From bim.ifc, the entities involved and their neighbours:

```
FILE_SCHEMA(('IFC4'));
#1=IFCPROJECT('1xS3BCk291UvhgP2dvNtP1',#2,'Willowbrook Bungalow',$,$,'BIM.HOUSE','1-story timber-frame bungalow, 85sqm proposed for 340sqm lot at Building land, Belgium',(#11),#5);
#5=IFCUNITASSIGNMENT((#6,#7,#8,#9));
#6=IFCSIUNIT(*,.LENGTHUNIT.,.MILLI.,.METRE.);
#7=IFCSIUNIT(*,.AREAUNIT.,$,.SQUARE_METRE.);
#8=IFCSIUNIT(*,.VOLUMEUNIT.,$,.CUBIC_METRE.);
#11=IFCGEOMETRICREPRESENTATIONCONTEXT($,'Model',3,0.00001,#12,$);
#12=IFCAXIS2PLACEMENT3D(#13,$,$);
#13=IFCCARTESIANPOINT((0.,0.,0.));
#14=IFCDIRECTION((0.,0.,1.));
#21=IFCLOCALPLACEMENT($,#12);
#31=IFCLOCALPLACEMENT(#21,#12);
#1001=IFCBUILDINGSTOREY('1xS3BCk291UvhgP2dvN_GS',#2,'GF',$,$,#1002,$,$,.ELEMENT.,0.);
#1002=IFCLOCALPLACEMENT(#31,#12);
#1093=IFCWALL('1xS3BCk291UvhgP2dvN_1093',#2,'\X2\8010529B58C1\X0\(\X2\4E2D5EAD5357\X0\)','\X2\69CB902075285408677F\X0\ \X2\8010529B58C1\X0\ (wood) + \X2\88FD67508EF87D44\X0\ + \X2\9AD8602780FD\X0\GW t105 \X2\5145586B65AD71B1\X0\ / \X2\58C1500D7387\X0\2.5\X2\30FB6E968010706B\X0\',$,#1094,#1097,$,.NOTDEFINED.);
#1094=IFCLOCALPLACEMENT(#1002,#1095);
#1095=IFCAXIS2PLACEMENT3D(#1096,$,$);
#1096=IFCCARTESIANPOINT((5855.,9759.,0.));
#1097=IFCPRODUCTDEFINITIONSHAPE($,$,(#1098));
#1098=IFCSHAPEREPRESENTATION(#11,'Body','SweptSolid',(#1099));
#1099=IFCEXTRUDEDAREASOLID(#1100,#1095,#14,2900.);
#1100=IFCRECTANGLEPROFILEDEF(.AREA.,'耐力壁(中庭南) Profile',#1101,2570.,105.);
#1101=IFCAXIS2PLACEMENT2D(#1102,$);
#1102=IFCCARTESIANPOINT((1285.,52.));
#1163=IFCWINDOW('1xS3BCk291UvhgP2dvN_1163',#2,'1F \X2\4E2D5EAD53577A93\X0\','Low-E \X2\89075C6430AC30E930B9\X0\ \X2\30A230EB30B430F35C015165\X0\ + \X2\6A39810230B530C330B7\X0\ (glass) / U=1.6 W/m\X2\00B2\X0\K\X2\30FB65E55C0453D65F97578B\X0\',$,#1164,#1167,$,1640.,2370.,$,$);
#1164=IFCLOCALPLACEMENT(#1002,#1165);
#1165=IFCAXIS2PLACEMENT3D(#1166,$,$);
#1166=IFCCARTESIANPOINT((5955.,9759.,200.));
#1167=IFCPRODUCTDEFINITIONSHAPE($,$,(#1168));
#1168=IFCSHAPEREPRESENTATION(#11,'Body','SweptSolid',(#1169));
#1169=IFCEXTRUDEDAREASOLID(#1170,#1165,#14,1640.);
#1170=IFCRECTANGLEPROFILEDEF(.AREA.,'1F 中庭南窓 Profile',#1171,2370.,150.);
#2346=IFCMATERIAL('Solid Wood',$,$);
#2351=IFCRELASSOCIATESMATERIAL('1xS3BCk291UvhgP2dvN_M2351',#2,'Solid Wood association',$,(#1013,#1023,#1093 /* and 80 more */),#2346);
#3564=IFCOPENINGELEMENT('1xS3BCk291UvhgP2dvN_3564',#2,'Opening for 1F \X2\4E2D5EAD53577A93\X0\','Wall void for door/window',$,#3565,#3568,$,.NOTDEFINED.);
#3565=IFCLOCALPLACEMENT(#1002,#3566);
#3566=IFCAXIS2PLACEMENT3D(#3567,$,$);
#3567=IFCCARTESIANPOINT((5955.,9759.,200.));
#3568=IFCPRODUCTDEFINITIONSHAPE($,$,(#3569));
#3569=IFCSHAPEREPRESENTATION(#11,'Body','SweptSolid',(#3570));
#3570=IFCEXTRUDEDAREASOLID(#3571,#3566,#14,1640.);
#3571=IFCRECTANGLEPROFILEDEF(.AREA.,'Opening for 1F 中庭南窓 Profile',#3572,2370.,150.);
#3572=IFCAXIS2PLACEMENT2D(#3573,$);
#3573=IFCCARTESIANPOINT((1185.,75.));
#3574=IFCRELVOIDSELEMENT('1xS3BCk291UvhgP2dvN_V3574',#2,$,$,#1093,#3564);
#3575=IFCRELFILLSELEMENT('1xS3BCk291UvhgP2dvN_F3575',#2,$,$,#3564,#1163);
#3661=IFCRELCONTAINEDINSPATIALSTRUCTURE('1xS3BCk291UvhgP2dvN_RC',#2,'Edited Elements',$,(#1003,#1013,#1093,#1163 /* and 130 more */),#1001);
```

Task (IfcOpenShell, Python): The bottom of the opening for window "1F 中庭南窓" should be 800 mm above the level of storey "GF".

```python
import numpy as np
import ifcopenshell
import ifcopenshell.api.geometry
import ifcopenshell.geom
import ifcopenshell.util.element
import ifcopenshell.util.placement
import ifcopenshell.util.shape
import ifcopenshell.util.unit

model = ifcopenshell.open("bim.ifc")
unit_scale = ifcopenshell.util.unit.calculate_unit_scale(model)

window = model.by_guid("1xS3BCk291UvhgP2dvN_1163")
opening = window.FillsVoids[0].RelatingOpeningElement
storey = ifcopenshell.util.element.get_container(window, ifc_class="IfcBuildingStorey")
level = ifcopenshell.util.placement.get_local_placement(storey.ObjectPlacement)[2, 3]

# The opening's origin need not be at the sill, so measure its lowest point.
shape = ifcopenshell.geom.create_shape(ifcopenshell.geom.settings(), opening)
bottom = ifcopenshell.util.shape.get_shape_bottom_elevation(shape, shape.geometry) / unit_scale
dz = level + 800.0 - bottom

shift = np.array([0.0, 0.0, dz])
# The window is not placed relative to its opening, so move both.
for product in (opening, window):
    matrix = ifcopenshell.util.placement.get_local_placement(product.ObjectPlacement)
    matrix[:3, 3] += shift
    ifcopenshell.api.geometry.edit_object_placement(model, product=product, matrix=matrix, is_si=False)

print(f"moved by {dz * unit_scale:+.3f} m")

model.write("bim-out.ifc")
```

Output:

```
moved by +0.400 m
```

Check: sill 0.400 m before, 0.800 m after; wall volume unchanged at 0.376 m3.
